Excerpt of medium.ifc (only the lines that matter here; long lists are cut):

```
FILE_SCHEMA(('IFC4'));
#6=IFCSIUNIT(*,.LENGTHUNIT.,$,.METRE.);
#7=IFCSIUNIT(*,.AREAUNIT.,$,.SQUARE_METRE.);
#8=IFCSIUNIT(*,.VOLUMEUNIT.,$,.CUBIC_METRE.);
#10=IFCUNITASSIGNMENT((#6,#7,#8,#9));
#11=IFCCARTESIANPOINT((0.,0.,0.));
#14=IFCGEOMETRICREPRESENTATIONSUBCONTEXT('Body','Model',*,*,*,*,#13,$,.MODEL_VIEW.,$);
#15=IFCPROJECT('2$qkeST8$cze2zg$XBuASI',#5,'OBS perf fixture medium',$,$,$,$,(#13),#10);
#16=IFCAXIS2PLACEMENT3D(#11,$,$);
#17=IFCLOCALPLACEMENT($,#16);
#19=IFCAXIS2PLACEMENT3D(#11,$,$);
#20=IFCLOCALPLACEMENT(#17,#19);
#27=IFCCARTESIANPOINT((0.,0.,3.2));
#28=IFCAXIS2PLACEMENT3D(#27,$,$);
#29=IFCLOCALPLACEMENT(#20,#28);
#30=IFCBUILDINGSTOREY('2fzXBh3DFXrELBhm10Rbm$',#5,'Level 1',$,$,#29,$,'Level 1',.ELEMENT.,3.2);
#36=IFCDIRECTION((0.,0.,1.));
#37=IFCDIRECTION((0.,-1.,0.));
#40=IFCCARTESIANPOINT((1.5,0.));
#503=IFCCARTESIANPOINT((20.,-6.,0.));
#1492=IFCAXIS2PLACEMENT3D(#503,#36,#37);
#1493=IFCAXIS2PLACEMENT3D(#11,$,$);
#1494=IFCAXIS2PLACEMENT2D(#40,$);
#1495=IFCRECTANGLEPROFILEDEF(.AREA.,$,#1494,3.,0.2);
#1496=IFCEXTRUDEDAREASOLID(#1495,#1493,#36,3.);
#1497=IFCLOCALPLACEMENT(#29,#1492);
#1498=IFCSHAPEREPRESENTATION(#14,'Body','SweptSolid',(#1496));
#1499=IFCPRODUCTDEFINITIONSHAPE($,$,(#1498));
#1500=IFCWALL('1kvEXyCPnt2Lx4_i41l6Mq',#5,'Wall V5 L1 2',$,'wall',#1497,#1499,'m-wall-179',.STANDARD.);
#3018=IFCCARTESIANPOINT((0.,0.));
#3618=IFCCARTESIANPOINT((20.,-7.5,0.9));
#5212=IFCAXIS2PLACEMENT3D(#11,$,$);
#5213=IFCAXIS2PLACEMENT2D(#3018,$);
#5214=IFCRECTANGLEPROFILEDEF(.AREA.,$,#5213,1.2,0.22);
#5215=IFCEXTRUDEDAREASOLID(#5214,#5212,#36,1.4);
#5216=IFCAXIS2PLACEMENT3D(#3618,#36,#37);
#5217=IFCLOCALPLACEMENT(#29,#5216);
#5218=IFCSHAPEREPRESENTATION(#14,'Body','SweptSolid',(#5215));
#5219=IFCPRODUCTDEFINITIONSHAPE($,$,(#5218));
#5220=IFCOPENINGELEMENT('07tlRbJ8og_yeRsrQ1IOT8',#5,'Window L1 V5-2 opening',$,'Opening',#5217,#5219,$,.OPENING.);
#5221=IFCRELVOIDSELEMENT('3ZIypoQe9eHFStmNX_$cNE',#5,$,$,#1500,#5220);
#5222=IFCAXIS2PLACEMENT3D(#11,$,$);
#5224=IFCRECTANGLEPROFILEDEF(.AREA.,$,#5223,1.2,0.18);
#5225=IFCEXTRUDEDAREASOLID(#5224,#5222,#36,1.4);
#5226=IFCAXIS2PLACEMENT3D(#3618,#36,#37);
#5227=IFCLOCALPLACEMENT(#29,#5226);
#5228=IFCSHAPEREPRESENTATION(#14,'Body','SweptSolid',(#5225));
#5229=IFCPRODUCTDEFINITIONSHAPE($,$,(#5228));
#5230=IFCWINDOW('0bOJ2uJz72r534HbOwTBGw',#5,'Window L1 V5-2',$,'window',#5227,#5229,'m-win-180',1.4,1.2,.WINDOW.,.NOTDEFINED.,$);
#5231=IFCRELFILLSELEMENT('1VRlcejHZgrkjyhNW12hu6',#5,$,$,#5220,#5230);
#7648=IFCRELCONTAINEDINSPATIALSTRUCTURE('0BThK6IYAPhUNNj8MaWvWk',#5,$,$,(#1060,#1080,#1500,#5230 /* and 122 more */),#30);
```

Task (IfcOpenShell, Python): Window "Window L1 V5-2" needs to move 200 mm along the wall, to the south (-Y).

```python
import ifcopenshell
import ifcopenshell.api.geometry
import ifcopenshell.util.placement
import ifcopenshell.util.unit

model = ifcopenshell.open("medium.ifc")
unit_scale = ifcopenshell.util.unit.calculate_unit_scale(model)

window = model.by_guid("0bOJ2uJz72r534HbOwTBGw")
opening = window.FillsVoids[0].RelatingOpeningElement
wall = opening.VoidsElements[0].RelatingBuildingElement

wall_matrix = ifcopenshell.util.placement.get_local_placement(wall.ObjectPlacement)
shift = wall_matrix[:3, 0] * 0.2 / unit_scale
before = ifcopenshell.util.placement.get_local_placement(window.ObjectPlacement)[:3, 3].copy()

# The window is not placed relative to its opening, so move both.
for product in (opening, window):
    matrix = ifcopenshell.util.placement.get_local_placement(product.ObjectPlacement)
    matrix[:3, 3] += shift
    ifcopenshell.api.geometry.edit_object_placement(model, product=product, matrix=matrix, is_si=False)

after = ifcopenshell.util.placement.get_local_placement(window.ObjectPlacement)[:3, 3]
print("window moved by", (after - before).round(3) + 0.0)

model.write("medium_edited.ifc")
```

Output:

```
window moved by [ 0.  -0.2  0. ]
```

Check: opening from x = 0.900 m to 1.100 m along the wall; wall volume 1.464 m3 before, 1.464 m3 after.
